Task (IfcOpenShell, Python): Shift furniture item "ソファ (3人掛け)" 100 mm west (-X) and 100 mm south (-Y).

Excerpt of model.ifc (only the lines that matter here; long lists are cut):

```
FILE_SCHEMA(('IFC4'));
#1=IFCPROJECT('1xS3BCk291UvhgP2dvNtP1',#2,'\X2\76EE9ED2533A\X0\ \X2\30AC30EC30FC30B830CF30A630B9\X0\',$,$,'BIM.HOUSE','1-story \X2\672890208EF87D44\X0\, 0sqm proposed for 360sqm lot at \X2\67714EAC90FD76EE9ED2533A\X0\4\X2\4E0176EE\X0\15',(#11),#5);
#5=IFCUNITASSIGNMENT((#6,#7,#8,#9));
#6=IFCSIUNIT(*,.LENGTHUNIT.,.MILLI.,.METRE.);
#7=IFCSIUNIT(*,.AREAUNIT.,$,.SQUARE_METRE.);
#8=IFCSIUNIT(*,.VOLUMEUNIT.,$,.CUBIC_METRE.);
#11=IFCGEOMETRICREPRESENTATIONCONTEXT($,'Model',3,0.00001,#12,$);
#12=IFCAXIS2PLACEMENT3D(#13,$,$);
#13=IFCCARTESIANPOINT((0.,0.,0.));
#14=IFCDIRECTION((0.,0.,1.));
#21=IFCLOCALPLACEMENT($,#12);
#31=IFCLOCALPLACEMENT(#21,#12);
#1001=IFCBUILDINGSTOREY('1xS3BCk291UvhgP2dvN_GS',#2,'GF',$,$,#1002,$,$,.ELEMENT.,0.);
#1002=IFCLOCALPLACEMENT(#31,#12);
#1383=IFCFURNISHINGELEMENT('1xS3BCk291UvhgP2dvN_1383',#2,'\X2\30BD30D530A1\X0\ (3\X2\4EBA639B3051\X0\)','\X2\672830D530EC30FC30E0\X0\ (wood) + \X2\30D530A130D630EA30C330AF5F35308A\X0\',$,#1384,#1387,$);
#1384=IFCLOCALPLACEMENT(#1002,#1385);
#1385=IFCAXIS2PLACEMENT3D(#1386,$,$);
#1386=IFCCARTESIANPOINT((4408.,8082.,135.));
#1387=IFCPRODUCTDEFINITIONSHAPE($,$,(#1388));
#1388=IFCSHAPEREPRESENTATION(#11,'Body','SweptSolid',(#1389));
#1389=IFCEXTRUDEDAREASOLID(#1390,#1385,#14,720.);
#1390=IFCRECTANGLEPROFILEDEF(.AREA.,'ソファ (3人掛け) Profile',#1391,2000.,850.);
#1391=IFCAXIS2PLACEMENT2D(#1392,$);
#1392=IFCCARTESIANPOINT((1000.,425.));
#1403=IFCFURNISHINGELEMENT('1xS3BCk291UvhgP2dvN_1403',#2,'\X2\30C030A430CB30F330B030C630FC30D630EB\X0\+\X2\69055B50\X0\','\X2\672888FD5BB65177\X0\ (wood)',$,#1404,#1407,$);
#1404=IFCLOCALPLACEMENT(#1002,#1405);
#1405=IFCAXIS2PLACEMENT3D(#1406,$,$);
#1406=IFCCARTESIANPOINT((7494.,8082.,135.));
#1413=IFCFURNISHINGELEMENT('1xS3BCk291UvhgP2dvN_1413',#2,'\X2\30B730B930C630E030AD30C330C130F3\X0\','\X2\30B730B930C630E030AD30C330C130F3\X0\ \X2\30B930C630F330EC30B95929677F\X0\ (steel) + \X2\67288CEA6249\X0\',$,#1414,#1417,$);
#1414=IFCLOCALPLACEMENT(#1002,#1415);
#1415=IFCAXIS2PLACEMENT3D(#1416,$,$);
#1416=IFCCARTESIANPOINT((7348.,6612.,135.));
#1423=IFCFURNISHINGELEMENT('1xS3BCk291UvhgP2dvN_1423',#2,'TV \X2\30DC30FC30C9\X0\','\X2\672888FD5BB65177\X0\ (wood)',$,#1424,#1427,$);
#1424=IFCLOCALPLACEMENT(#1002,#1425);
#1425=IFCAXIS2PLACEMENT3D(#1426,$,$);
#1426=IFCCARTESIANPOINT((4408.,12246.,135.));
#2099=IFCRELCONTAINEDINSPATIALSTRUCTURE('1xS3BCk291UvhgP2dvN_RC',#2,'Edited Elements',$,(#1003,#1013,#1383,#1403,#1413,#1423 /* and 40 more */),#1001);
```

```python
import ifcopenshell
import ifcopenshell.api.geometry
import ifcopenshell.util.placement

model = ifcopenshell.open("model.ifc")

item = model.by_guid("1xS3BCk291UvhgP2dvN_1383")
matrix = ifcopenshell.util.placement.get_local_placement(item.ObjectPlacement)
matrix[0, 3] -= 100.0
matrix[1, 3] -= 100.0
ifcopenshell.api.geometry.edit_object_placement(model, product=item, matrix=matrix, is_si=False)

print(ifcopenshell.util.placement.get_local_placement(item.ObjectPlacement).round(3) + 0.0)

model.write("model-out.ifc")
```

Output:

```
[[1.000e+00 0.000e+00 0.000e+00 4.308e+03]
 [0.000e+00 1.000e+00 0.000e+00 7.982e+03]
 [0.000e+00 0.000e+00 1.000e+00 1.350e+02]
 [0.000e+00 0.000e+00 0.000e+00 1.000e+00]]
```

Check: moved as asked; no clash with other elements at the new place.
